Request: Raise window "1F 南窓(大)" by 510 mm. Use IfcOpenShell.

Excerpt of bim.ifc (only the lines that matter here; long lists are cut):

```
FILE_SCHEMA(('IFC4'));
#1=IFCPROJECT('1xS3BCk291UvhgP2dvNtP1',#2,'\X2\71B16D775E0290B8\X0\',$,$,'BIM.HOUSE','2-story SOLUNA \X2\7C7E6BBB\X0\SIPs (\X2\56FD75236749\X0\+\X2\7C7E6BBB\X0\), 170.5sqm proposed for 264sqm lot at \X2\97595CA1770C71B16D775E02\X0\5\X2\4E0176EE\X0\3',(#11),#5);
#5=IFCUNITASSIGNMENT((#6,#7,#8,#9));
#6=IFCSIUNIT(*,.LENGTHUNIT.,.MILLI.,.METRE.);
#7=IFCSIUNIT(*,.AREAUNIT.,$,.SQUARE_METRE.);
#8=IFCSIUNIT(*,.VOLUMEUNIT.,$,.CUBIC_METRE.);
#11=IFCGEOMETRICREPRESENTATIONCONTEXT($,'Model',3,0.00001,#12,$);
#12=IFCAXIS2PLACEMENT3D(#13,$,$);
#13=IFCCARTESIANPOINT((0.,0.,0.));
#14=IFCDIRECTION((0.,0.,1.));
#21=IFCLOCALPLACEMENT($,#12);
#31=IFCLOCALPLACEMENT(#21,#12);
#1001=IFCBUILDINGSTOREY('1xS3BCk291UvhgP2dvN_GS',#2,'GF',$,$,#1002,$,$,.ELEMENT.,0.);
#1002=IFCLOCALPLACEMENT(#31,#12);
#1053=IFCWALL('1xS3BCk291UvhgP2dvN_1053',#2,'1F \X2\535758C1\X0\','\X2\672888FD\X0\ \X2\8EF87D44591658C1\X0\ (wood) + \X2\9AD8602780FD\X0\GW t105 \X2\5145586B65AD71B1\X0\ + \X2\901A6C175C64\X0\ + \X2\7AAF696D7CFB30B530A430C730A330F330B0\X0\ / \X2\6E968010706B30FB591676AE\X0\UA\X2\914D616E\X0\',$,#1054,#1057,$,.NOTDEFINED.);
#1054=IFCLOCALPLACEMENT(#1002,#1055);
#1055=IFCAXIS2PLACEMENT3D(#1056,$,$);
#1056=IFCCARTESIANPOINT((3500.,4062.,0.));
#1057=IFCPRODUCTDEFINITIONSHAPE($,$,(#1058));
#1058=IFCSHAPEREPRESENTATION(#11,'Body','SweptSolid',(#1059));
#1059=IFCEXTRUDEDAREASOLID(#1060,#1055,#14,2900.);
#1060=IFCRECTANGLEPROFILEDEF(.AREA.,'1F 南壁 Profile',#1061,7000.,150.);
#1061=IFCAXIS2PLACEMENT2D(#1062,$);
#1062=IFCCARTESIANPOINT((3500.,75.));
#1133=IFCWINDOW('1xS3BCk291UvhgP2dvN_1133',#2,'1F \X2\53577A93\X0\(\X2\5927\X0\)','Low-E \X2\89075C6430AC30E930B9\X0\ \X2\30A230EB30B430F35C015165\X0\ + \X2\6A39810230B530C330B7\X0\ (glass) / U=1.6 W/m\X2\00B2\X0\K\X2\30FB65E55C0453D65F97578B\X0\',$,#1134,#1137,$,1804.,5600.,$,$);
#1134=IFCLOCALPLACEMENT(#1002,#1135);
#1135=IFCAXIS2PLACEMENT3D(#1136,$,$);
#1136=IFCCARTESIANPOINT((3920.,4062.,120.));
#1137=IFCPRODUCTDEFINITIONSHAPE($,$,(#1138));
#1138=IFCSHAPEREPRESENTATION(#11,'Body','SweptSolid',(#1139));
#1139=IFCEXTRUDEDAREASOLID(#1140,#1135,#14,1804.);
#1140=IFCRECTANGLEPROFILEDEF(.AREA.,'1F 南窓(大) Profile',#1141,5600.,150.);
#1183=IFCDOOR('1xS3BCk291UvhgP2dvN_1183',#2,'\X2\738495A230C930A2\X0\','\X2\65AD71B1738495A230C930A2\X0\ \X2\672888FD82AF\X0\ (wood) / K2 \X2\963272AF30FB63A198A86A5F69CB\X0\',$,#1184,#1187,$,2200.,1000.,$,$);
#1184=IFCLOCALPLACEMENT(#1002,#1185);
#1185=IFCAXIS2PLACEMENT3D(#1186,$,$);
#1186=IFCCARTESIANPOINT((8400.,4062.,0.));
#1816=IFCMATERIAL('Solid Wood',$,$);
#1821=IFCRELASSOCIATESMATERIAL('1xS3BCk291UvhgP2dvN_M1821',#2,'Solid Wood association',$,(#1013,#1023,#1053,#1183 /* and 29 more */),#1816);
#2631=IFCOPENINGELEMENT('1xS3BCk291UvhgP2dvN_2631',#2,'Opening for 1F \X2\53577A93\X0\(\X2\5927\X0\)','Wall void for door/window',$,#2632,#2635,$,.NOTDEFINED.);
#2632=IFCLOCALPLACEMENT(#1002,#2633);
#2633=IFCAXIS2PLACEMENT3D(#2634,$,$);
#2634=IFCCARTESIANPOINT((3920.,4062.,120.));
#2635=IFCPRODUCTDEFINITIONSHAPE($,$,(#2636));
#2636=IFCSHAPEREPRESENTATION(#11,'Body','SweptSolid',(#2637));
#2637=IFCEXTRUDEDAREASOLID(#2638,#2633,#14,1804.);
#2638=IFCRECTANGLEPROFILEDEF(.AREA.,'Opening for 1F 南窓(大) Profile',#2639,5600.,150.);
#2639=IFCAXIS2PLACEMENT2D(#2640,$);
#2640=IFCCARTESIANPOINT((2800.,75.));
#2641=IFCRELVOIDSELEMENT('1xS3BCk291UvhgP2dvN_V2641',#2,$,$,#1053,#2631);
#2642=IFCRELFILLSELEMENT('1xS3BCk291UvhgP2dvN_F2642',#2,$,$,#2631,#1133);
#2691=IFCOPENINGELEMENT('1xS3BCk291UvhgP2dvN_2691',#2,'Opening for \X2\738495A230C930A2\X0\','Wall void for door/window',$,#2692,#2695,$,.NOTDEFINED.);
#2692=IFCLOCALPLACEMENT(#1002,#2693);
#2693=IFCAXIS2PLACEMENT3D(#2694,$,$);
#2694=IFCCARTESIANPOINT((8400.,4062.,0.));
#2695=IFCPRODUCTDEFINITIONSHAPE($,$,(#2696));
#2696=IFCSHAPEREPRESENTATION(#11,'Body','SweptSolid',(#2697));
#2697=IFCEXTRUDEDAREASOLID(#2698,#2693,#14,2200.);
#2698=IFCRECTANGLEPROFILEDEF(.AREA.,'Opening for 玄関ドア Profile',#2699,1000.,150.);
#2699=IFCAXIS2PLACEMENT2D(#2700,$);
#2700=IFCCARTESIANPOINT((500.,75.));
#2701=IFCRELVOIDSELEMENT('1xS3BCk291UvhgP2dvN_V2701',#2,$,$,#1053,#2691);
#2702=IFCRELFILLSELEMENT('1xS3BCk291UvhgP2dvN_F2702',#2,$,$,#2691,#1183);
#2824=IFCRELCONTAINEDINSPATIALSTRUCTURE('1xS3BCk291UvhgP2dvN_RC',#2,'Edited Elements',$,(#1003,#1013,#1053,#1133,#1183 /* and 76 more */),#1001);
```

```python
import numpy as np
import ifcopenshell
import ifcopenshell.api.geometry
import ifcopenshell.util.placement
import ifcopenshell.util.unit

model = ifcopenshell.open("bim.ifc")
unit_scale = ifcopenshell.util.unit.calculate_unit_scale(model)

window = model.by_guid("1xS3BCk291UvhgP2dvN_1133")
opening = window.FillsVoids[0].RelatingOpeningElement
dz = 0.51 / unit_scale

shift = np.array([0.0, 0.0, dz])
# The window is not placed relative to its opening, so move both.
for product in (opening, window):
    matrix = ifcopenshell.util.placement.get_local_placement(product.ObjectPlacement)
    matrix[:3, 3] += shift
    ifcopenshell.api.geometry.edit_object_placement(model, product=product, matrix=matrix, is_si=False)

print(f"moved by {dz * unit_scale:+.3f} m")

model.write("bim_rev.ifc")
```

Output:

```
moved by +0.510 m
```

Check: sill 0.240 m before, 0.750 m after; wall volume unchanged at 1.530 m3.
